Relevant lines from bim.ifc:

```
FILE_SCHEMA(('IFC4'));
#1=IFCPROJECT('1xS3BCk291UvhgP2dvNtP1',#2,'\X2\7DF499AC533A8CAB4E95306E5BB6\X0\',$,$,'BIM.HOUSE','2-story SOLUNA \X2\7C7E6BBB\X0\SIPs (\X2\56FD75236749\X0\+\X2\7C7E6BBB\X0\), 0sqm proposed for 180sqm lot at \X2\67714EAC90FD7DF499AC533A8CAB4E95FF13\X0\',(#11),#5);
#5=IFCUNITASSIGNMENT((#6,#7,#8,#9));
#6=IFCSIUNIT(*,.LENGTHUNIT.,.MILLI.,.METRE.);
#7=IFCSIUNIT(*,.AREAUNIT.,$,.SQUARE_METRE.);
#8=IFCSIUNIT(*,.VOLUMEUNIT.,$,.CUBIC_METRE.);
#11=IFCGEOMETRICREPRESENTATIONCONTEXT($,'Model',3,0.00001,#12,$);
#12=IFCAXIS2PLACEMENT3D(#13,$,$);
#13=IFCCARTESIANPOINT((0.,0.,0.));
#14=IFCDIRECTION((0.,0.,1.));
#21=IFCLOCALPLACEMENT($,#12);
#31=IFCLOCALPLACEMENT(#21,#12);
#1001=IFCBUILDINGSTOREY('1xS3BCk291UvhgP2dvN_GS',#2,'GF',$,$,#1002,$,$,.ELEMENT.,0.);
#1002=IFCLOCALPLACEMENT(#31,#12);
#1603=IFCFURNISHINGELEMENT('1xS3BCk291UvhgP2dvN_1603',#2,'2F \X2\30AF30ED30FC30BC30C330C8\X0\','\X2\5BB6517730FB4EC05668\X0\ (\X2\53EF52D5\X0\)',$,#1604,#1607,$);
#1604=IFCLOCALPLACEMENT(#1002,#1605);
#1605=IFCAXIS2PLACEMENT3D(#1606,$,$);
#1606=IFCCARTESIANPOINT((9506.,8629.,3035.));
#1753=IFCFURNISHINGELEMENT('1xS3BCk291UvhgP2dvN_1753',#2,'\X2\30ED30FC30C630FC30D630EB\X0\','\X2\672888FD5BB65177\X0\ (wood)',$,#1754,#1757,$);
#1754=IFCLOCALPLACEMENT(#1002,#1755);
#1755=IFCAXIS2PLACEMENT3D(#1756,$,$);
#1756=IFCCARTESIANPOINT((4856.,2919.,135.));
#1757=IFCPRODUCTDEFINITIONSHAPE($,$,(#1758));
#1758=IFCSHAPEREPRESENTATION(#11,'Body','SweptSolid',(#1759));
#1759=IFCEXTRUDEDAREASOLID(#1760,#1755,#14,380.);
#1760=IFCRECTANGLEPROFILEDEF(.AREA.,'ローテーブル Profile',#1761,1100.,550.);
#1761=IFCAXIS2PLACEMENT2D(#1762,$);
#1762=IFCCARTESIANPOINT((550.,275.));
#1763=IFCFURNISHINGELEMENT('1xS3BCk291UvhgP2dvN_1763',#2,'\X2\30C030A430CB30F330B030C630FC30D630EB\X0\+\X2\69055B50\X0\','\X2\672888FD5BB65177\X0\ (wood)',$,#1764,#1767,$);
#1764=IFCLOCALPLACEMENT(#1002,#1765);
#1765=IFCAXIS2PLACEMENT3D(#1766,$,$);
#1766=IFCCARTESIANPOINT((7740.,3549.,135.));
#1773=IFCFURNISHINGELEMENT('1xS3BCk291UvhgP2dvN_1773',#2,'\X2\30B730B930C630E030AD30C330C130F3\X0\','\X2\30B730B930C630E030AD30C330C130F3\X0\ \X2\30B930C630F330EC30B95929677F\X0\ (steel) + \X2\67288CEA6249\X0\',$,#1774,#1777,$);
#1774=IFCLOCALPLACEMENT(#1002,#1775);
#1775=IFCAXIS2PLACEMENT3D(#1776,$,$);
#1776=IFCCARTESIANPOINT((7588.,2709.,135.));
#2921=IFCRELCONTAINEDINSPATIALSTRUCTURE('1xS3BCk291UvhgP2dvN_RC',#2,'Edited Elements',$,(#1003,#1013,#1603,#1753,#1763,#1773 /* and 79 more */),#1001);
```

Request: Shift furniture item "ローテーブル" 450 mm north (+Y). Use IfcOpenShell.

```python
import ifcopenshell
import ifcopenshell.api.geometry
import ifcopenshell.util.placement

model = ifcopenshell.open("bim.ifc")

item = model.by_id(1753)
matrix = ifcopenshell.util.placement.get_local_placement(item.ObjectPlacement)
matrix[1, 3] += 450.0
ifcopenshell.api.geometry.edit_object_placement(model, product=item, matrix=matrix, is_si=False)

print(ifcopenshell.util.placement.get_local_placement(item.ObjectPlacement).round(3) + 0.0)

model.write("bim-out.ifc")
```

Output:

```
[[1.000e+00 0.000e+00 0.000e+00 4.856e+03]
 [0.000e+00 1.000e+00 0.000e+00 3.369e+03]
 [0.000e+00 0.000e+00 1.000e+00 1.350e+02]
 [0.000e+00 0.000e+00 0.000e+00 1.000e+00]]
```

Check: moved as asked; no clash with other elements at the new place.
